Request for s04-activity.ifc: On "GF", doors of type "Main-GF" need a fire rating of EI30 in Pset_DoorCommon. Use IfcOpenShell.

First a look at what the model holds.

```python
import ifcopenshell
import ifcopenshell.util.element

model = ifcopenshell.open("s04-activity.ifc")
print(model.schema)
storey = next(s for s in model.by_type("IfcBuildingStorey") if s.Name == "GF")
doors = [e for e in ifcopenshell.util.element.get_decomposition(storey) if e.is_a("IfcDoor")]
seen = {}
for e in doors:
    element_type = ifcopenshell.util.element.get_type(e)
    key = (element_type.Name if element_type != e and element_type else None, ifcopenshell.util.element.get_pset(e, "Pset_DoorCommon", "FireRating"))
    seen[key] = seen.get(key, 0) + 1
for (name, value), count in sorted(seen.items(), key=str):
    print(count, "x", name, "|", value)
```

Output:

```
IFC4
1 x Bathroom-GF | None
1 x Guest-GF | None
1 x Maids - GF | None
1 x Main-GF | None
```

```python
import ifcopenshell
import ifcopenshell.api.pset
import ifcopenshell.util.element

model = ifcopenshell.open("s04-activity.ifc")

storey = next(s for s in model.by_type("IfcBuildingStorey") if s.Name == "GF")
doors = [e for e in ifcopenshell.util.element.get_decomposition(storey) if e.is_a("IfcDoor")]

count = 0
for e in doors:
    element_type = ifcopenshell.util.element.get_type(e)
    if element_type in (None, e) or element_type.Name != "Main-GF":
        continue
    # add_pset returns the element's existing set when there is one.
    pset = ifcopenshell.api.pset.add_pset(model, product=e, name="Pset_DoorCommon")
    ifcopenshell.api.pset.edit_pset(model, pset=pset, properties={"FireRating": "EI30"})
    count += 1

print(count, "doors updated")

model.write("s04-activity_updated.ifc")
```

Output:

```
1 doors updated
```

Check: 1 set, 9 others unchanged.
